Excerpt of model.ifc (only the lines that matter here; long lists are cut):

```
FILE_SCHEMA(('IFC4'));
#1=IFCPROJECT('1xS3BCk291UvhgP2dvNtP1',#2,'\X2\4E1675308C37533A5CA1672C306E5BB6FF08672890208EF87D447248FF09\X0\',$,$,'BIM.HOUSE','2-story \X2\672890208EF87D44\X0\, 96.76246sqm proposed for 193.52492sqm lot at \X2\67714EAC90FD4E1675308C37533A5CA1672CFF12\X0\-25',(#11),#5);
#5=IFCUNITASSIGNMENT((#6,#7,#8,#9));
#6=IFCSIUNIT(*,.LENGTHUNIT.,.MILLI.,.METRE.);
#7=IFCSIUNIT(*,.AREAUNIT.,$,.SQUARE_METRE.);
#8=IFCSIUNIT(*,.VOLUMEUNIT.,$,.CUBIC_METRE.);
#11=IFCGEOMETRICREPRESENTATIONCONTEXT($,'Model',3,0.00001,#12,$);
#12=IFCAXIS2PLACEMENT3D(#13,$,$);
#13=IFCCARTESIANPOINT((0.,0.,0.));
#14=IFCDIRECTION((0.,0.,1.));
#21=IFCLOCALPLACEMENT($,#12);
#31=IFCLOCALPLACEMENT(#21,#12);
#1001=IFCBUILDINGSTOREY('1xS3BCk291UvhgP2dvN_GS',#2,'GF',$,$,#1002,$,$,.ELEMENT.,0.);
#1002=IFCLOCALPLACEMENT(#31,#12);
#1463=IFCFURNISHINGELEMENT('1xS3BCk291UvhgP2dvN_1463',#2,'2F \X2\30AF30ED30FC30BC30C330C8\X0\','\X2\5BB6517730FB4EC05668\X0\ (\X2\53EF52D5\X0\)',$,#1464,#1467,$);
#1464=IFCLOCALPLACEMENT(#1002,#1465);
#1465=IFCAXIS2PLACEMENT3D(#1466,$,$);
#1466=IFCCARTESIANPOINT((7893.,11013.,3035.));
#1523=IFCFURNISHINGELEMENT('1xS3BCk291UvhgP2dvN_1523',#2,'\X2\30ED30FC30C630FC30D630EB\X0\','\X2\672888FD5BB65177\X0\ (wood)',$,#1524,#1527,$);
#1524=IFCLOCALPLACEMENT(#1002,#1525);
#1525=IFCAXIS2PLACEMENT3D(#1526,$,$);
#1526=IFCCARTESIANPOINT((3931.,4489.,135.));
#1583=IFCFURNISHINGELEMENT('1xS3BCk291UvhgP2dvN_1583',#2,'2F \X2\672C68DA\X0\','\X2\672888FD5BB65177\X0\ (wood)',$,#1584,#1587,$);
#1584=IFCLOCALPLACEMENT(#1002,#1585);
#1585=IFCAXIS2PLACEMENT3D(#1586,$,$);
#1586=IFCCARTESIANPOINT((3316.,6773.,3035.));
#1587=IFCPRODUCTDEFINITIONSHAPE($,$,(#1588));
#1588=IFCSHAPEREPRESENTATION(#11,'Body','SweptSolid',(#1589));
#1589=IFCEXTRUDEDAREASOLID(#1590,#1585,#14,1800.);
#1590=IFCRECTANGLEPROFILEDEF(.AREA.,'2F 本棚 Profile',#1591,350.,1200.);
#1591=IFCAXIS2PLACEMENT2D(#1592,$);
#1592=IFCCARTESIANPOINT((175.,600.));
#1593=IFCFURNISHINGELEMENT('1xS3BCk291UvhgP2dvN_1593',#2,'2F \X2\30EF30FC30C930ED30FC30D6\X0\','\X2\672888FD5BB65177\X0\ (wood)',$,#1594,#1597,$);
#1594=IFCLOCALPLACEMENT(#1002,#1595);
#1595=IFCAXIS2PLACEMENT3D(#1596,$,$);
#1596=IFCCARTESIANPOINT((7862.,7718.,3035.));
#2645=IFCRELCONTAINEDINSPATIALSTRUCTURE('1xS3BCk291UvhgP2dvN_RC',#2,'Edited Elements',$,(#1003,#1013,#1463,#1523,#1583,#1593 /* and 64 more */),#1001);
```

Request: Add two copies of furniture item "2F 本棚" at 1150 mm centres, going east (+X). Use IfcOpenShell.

```python
import numpy as np
import ifcopenshell
import ifcopenshell.api.geometry
import ifcopenshell.api.root
import ifcopenshell.util.element
import ifcopenshell.util.placement

model = ifcopenshell.open("model.ifc")


def reuse_history(source, copy):
    """copy_class also copies each property set's owner history, people and application; keep the originals."""
    for rel in copy.IsDefinedBy:
        if rel.is_a("IfcRelDefinesByProperties") and (history := rel.RelatingPropertyDefinition.OwnerHistory):
            rel.RelatingPropertyDefinition.OwnerHistory = source.OwnerHistory
            ifcopenshell.util.element.remove_deep2(model, history)


source = model.by_guid("1xS3BCk291UvhgP2dvN_1583")
base = ifcopenshell.util.placement.get_local_placement(source.ObjectPlacement)
step = np.array([1.0, 0.0, 0.0]) * 1150.0

for i in range(1, 3):
    copy = ifcopenshell.api.root.copy_class(model, product=source)
    copy.Representation = ifcopenshell.util.element.copy_deep(
        model, source.Representation, exclude=["IfcGeometricRepresentationContext", "IfcRepresentationMap"]
    )
    reuse_history(source, copy)
    matrix = base.copy()
    matrix[:3, 3] += i * step
    print("added at", matrix[:3, 3].round(3) + 0.0)
    ifcopenshell.api.geometry.edit_object_placement(model, product=copy, matrix=matrix, is_si=False)

model.write("model_edited.ifc")
```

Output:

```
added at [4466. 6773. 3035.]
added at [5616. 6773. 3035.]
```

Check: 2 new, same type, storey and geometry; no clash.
